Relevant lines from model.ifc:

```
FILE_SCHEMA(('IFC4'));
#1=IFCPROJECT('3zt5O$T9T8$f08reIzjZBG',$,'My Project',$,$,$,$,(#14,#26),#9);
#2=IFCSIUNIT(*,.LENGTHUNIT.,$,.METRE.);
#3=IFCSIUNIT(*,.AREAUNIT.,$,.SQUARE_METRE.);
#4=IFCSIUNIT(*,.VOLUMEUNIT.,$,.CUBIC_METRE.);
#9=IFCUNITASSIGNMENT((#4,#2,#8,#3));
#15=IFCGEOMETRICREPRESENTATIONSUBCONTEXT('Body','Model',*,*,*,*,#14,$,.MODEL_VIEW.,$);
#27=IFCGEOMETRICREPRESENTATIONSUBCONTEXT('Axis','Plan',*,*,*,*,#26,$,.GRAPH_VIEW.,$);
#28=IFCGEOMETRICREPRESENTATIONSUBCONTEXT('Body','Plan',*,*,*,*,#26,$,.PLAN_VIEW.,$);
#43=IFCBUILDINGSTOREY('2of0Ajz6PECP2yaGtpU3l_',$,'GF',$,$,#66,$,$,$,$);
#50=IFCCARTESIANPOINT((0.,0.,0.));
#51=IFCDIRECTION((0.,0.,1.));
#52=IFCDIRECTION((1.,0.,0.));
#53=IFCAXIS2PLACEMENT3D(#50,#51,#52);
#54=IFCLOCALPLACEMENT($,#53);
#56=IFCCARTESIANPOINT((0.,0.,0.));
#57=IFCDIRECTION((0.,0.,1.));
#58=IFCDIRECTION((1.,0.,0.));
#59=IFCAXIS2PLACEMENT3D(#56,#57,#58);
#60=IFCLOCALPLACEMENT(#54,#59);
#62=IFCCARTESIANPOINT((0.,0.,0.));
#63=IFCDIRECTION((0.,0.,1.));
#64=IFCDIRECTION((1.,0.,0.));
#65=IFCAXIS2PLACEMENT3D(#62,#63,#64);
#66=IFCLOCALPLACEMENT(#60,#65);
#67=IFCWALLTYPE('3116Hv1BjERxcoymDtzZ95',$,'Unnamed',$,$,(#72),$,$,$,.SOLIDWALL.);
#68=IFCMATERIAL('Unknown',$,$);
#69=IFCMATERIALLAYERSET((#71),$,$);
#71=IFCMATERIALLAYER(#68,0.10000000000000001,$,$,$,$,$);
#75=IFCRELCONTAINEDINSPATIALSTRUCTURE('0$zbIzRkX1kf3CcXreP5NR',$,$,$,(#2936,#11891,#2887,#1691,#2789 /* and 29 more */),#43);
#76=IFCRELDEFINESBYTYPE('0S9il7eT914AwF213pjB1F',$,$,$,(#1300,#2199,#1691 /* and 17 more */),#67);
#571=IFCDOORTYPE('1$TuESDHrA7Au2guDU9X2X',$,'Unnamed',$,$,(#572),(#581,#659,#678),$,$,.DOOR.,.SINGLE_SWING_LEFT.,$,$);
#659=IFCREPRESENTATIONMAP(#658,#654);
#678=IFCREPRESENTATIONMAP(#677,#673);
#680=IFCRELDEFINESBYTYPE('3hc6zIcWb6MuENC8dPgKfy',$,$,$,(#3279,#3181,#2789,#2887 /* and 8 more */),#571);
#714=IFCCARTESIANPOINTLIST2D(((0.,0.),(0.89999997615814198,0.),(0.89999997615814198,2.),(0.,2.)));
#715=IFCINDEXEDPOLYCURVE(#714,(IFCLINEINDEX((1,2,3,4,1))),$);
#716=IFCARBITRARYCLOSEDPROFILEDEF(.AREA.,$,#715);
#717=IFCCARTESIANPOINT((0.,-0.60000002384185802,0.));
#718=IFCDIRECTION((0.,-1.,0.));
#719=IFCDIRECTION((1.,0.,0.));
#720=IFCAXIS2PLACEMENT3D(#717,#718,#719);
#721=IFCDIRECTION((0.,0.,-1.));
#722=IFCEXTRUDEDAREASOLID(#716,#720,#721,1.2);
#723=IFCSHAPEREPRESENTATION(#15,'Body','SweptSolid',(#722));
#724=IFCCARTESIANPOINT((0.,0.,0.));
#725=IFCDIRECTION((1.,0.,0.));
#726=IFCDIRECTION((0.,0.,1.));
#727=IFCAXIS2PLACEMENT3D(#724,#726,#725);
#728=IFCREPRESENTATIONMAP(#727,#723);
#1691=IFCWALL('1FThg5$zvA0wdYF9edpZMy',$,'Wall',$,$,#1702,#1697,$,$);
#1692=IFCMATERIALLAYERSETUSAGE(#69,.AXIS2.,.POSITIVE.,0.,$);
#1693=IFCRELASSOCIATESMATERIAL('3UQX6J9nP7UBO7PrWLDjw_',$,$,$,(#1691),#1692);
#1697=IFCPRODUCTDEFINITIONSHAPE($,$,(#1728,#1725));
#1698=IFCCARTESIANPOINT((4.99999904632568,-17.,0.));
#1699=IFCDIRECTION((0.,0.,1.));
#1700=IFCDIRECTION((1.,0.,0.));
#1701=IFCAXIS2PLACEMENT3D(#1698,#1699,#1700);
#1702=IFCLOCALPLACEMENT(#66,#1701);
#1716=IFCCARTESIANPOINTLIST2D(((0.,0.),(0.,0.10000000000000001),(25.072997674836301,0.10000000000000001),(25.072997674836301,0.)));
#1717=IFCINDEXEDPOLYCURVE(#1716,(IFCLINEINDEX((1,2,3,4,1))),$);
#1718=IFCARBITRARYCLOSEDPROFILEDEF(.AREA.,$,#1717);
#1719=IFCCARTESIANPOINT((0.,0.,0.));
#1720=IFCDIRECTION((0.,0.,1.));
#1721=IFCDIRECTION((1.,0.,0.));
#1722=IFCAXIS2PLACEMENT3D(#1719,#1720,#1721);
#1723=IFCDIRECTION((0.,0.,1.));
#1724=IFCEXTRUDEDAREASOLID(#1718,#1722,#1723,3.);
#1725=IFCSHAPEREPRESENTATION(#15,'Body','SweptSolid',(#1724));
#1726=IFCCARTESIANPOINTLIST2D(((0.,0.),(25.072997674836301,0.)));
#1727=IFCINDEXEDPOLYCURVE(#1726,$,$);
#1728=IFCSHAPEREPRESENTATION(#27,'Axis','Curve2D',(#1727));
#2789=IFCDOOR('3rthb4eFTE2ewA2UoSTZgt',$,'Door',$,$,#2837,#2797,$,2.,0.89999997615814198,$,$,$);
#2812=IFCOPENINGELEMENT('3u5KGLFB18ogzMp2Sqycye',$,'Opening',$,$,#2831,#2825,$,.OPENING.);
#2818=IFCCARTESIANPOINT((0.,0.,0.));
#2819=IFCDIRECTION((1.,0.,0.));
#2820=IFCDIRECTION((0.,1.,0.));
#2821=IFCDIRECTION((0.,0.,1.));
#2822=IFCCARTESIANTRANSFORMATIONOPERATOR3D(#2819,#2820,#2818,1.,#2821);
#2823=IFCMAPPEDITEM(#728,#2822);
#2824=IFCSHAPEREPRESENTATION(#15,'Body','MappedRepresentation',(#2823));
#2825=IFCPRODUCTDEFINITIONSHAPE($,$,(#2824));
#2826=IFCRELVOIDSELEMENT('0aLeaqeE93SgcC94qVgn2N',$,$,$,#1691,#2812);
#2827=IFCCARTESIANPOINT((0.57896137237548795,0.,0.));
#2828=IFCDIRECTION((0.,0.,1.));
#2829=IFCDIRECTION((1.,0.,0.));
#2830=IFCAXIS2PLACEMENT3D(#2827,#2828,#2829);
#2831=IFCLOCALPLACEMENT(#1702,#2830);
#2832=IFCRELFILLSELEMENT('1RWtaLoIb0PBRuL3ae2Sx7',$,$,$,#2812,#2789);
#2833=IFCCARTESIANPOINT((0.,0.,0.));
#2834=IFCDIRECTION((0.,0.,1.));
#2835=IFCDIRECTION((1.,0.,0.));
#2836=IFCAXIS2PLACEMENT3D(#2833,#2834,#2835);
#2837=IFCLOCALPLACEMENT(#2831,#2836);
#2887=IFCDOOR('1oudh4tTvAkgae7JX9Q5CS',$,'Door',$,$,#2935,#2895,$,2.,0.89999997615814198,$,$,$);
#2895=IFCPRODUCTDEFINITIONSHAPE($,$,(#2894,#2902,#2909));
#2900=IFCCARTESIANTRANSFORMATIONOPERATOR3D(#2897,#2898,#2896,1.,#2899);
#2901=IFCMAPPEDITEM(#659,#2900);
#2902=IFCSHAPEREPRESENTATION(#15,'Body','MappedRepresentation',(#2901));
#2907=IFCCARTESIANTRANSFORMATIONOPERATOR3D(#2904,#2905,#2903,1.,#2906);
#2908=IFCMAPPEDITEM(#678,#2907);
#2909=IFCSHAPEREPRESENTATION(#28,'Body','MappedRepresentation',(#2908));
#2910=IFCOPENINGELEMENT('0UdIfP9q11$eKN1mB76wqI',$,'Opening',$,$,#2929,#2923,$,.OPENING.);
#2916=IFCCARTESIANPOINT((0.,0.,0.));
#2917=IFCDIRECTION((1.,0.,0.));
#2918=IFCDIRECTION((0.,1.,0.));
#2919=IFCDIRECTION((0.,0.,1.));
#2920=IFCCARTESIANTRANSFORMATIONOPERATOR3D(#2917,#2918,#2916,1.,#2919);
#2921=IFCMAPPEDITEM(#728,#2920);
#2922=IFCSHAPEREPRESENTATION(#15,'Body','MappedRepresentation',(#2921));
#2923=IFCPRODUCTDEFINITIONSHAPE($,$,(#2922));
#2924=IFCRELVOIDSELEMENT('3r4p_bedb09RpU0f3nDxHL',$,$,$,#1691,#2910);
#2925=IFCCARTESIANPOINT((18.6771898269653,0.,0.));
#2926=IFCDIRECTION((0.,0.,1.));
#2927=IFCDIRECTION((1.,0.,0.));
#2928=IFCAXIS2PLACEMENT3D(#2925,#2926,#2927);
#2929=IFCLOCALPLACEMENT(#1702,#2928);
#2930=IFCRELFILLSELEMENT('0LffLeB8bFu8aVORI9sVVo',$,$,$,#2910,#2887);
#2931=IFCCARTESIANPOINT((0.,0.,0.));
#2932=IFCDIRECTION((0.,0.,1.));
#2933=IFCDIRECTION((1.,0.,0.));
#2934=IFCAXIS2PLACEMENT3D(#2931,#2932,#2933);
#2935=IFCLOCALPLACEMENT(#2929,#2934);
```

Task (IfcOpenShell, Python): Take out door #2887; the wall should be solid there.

```python
import ifcopenshell
import ifcopenshell.api.feature
import ifcopenshell.api.root
import ifcopenshell.geom
import ifcopenshell.util.shape

model = ifcopenshell.open("model.ifc")
settings = ifcopenshell.geom.settings()


def volume(element):
    """Net volume in cubic metres, openings subtracted."""
    shape = ifcopenshell.geom.create_shape(settings, element)
    return ifcopenshell.util.shape.get_volume(shape.geometry)


door = model.by_id(2887)
opening = door.FillsVoids[0].RelatingOpeningElement
wall = opening.VoidsElements[0].RelatingBuildingElement
before = volume(wall)

ifcopenshell.api.root.remove_product(model, product=door)
ifcopenshell.api.feature.remove_feature(model, feature=opening)

after = volume(wall)

print(f"wall volume {before:.3f} -> {after:.3f} m3")

model.write("model-out.ifc")
```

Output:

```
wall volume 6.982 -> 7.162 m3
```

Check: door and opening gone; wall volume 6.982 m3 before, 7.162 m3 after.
